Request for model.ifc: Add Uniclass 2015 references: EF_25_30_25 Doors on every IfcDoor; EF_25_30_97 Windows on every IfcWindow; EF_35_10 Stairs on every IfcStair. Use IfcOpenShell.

First a look at what the model holds.

```python
import ifcopenshell

model = ifcopenshell.open("model.ifc")
print(model.schema)
print("classifications:", [c.Name for c in model.by_type("IfcClassification")])
for ifc_class in ("IfcDoor", "IfcRoof", "IfcStair", "IfcWall", "IfcWindow"):
    print(ifc_class, len(model.by_type(ifc_class)))
```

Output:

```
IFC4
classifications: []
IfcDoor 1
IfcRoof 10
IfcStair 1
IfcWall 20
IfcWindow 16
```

```python
import ifcopenshell
import ifcopenshell.api.classification

model = ifcopenshell.open("model.ifc")

system = ifcopenshell.api.classification.add_classification(model, classification="Uniclass 2015")

codes = {
    "IfcDoor": ("EF_25_30_25", "Doors"),
    "IfcWindow": ("EF_25_30_97", "Windows"),
    "IfcStair": ("EF_35_10", "Stairs"),
}
for ifc_class, (code, name) in codes.items():
    products = model.by_type(ifc_class)
    ifcopenshell.api.classification.add_reference(
        model, products=products, classification=system, identification=code, name=name
    )
    print(code, len(products))

model.write("model_v2.ifc")
```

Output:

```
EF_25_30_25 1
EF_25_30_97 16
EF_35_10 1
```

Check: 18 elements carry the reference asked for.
